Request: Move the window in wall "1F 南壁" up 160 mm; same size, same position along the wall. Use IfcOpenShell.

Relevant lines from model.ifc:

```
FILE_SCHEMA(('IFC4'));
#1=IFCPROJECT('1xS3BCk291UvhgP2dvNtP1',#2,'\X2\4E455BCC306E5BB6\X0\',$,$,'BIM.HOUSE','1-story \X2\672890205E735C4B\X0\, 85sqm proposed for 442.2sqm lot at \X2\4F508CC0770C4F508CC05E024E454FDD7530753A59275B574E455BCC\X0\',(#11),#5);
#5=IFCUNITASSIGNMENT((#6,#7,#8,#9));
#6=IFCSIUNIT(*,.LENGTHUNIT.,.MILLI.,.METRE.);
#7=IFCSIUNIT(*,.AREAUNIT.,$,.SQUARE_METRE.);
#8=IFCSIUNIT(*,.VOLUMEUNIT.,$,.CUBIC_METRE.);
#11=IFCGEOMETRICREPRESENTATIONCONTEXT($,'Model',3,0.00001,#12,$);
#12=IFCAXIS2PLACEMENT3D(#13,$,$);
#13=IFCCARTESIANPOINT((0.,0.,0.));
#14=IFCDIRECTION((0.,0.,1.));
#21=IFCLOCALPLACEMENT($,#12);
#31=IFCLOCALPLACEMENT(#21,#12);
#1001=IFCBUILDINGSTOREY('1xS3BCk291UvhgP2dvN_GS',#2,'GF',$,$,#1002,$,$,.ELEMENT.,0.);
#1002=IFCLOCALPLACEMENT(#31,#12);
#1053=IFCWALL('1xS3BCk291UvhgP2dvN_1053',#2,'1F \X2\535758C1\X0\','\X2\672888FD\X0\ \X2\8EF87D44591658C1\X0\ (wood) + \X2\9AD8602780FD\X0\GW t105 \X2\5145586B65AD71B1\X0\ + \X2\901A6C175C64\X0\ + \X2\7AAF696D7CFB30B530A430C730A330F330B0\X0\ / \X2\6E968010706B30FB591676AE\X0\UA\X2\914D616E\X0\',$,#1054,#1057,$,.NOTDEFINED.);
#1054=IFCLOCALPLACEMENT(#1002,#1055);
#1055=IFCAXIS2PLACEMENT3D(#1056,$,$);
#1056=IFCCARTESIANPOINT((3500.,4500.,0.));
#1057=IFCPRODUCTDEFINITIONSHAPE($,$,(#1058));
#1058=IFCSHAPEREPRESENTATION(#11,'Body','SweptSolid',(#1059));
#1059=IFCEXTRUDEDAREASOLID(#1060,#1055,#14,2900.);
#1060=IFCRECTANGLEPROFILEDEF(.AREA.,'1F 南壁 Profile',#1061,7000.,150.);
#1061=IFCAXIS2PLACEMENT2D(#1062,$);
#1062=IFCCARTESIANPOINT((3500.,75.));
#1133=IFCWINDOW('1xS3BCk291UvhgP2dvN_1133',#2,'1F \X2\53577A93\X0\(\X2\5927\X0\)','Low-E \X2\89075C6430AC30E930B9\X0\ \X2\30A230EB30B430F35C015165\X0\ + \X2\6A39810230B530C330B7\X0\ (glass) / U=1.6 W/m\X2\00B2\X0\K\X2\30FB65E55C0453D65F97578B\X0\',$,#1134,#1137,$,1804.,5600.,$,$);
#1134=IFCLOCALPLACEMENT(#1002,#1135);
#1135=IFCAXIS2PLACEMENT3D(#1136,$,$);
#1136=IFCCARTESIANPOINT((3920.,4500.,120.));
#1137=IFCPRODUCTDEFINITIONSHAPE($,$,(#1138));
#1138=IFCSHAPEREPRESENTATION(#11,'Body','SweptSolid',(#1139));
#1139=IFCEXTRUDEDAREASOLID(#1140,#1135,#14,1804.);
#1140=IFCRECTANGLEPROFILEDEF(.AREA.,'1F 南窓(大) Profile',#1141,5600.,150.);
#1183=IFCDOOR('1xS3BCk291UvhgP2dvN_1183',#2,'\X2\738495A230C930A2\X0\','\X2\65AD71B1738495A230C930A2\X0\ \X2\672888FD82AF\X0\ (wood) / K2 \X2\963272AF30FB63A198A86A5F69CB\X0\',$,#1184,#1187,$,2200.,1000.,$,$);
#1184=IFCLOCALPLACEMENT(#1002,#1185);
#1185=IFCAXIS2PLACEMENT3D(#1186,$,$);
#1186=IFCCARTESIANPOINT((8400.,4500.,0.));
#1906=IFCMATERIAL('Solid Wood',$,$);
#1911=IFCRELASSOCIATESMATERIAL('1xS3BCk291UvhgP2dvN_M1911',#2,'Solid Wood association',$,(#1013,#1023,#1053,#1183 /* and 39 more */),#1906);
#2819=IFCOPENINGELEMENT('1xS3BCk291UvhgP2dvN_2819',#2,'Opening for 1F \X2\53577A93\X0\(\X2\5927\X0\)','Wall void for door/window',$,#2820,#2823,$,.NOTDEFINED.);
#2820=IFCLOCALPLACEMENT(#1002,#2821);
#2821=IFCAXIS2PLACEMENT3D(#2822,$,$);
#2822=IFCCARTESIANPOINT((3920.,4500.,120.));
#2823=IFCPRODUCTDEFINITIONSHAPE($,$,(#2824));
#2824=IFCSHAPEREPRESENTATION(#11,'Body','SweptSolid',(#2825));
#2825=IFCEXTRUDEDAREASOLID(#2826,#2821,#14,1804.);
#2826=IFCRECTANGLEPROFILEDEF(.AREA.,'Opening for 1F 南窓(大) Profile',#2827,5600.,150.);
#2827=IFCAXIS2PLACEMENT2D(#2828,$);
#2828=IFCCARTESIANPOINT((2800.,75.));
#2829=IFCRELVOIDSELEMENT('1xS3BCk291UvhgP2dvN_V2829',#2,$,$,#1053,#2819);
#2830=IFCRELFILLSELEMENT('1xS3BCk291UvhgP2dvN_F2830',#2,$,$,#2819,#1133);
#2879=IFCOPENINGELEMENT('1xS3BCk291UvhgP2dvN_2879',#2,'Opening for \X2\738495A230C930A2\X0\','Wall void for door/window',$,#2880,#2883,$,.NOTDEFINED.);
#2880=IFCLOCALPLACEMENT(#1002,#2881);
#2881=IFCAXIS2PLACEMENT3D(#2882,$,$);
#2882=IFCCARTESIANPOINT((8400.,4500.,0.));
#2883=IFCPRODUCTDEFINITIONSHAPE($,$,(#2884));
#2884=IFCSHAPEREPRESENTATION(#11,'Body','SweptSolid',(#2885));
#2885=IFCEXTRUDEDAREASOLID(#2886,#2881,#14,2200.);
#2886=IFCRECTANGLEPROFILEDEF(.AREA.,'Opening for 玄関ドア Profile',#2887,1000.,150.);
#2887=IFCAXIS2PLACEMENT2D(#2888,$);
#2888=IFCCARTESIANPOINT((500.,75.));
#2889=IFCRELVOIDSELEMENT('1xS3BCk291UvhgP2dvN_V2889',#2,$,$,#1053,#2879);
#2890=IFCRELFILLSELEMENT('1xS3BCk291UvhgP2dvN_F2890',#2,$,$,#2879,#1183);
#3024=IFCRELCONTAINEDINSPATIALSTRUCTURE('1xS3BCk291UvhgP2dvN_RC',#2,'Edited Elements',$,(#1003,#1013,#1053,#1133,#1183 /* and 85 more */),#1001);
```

```python
import numpy as np
import ifcopenshell
import ifcopenshell.api.geometry
import ifcopenshell.util.placement
import ifcopenshell.util.unit

model = ifcopenshell.open("model.ifc")
unit_scale = ifcopenshell.util.unit.calculate_unit_scale(model)

window = model.by_guid("1xS3BCk291UvhgP2dvN_1133")
opening = window.FillsVoids[0].RelatingOpeningElement
dz = 0.16 / unit_scale

shift = np.array([0.0, 0.0, dz])
# The window is not placed relative to its opening, so move both.
for product in (opening, window):
    matrix = ifcopenshell.util.placement.get_local_placement(product.ObjectPlacement)
    matrix[:3, 3] += shift
    ifcopenshell.api.geometry.edit_object_placement(model, product=product, matrix=matrix, is_si=False)

print(f"moved by {dz * unit_scale:+.3f} m")

model.write("model_edited.ifc")
```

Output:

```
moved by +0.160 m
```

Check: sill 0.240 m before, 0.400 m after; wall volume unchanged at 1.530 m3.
